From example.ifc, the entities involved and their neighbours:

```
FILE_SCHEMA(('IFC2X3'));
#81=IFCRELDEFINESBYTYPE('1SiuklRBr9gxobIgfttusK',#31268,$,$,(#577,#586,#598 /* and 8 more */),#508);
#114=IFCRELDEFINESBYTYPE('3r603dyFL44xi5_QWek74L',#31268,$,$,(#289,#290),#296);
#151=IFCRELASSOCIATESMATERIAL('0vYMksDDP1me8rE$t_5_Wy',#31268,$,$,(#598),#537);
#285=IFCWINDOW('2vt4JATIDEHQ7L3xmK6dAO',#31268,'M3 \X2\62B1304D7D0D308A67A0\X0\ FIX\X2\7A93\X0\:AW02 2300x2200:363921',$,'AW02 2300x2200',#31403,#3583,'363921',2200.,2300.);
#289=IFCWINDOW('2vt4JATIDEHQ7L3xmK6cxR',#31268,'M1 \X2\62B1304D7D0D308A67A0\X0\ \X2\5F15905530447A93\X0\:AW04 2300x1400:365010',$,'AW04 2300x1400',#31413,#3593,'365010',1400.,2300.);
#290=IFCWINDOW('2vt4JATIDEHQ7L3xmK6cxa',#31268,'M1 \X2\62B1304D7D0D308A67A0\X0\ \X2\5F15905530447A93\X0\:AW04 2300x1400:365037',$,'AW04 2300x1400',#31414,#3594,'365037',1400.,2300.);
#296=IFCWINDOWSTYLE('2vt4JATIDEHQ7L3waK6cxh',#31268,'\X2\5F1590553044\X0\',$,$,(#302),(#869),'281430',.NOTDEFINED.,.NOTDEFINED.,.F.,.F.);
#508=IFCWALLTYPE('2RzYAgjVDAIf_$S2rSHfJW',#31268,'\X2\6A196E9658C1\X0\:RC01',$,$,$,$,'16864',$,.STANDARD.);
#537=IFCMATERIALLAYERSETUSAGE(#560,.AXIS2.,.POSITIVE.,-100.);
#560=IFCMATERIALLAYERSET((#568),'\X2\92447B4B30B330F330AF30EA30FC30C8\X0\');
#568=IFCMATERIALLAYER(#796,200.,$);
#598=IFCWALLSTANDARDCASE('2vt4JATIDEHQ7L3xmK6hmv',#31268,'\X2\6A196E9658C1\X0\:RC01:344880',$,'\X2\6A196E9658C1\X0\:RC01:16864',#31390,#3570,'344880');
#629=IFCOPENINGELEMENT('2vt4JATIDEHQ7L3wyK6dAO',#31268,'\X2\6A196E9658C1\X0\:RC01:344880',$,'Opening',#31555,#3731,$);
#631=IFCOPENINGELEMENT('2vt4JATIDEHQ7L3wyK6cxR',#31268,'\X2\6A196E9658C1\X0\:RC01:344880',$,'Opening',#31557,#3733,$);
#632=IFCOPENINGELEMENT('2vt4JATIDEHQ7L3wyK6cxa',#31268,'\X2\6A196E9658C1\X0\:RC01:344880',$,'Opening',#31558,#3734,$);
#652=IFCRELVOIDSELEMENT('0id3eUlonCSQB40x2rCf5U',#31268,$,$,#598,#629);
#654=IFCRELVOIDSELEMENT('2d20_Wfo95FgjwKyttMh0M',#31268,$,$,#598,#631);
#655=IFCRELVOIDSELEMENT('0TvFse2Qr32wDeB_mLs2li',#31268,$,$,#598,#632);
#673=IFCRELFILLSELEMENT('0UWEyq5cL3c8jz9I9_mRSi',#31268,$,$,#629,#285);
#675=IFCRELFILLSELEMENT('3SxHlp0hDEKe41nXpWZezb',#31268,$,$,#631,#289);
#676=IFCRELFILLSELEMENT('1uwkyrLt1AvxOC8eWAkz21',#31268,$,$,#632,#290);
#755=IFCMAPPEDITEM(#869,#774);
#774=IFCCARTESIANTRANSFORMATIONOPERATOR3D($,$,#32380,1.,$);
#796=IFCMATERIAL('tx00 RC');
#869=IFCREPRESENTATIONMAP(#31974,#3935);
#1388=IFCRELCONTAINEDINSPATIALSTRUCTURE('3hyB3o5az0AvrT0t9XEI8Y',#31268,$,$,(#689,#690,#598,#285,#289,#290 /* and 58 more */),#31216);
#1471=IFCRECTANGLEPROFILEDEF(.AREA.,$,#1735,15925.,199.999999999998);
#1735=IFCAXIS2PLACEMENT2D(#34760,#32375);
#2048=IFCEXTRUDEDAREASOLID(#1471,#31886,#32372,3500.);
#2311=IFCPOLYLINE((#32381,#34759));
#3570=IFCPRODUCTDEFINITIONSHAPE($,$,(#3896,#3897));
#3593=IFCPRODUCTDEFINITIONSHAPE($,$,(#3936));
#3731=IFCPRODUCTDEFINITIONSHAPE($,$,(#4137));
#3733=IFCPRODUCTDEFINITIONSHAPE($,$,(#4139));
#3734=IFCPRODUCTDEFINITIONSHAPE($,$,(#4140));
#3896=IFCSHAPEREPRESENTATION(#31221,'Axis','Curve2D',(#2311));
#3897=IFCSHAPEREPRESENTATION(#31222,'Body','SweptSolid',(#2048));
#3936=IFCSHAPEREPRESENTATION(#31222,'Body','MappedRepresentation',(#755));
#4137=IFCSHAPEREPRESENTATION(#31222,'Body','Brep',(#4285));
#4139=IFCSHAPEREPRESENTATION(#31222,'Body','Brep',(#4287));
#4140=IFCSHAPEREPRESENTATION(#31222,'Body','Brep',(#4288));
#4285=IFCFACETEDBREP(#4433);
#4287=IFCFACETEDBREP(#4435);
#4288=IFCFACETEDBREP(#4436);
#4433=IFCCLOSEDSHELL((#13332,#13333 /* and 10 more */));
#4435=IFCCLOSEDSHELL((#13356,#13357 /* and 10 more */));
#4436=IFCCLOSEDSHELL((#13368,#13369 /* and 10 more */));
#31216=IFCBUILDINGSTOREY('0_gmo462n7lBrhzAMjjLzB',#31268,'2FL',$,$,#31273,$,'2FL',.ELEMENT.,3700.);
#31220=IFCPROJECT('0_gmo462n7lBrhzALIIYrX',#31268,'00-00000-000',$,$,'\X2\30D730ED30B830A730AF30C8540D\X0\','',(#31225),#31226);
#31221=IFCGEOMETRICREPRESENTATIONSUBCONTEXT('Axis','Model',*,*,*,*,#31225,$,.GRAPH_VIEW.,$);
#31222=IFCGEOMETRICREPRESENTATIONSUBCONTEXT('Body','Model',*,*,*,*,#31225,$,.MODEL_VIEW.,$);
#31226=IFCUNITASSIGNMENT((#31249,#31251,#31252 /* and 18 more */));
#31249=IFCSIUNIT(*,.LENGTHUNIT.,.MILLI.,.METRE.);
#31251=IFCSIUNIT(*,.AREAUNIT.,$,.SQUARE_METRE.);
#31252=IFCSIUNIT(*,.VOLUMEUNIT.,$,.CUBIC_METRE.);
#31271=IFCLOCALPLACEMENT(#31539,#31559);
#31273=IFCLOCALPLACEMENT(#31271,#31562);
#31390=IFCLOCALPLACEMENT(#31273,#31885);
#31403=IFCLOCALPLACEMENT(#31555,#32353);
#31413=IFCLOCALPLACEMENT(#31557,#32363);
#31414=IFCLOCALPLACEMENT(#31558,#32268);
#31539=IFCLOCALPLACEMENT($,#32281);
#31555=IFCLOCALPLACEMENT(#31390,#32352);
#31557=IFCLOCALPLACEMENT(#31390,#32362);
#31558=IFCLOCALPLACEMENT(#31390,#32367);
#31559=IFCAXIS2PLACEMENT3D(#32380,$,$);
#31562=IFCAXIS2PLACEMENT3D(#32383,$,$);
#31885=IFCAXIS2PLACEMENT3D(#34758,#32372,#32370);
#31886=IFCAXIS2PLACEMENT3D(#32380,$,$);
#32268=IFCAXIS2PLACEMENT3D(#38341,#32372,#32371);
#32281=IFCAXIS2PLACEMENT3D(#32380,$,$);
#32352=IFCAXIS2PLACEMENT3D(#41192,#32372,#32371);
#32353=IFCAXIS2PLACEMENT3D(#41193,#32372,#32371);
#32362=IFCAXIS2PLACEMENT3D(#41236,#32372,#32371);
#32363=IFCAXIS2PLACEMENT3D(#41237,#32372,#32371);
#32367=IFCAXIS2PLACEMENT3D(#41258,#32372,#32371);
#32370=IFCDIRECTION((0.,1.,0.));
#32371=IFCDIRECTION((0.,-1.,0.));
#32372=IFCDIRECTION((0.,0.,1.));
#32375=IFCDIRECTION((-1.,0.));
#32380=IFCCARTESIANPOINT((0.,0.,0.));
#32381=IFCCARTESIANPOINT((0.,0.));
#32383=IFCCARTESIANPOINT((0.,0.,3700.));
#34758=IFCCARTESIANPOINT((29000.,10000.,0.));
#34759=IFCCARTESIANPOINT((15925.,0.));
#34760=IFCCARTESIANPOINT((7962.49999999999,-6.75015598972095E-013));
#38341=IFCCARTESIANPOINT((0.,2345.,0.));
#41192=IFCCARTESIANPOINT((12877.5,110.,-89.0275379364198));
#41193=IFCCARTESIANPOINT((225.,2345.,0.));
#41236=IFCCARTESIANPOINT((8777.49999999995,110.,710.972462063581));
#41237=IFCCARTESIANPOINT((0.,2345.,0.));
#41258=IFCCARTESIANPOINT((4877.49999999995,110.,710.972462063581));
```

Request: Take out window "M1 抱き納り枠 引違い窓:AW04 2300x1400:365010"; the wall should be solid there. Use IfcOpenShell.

```python
import ifcopenshell
import ifcopenshell.api.feature
import ifcopenshell.api.root
import ifcopenshell.geom
import ifcopenshell.util.shape

model = ifcopenshell.open("example.ifc")
settings = ifcopenshell.geom.settings()


def volume(element):
    """Net volume in cubic metres, openings subtracted."""
    shape = ifcopenshell.geom.create_shape(settings, element)
    return ifcopenshell.util.shape.get_volume(shape.geometry)


window = model.by_id(289)
opening = window.FillsVoids[0].RelatingOpeningElement
wall = opening.VoidsElements[0].RelatingBuildingElement
before = volume(wall)

ifcopenshell.api.root.remove_product(model, product=window)
ifcopenshell.api.feature.remove_feature(model, feature=opening)

after = volume(wall)

print(f"wall volume {before:.3f} -> {after:.3f} m3")

model.write("example-out.ifc")
```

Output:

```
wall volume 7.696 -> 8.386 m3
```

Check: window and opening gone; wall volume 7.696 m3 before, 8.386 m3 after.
